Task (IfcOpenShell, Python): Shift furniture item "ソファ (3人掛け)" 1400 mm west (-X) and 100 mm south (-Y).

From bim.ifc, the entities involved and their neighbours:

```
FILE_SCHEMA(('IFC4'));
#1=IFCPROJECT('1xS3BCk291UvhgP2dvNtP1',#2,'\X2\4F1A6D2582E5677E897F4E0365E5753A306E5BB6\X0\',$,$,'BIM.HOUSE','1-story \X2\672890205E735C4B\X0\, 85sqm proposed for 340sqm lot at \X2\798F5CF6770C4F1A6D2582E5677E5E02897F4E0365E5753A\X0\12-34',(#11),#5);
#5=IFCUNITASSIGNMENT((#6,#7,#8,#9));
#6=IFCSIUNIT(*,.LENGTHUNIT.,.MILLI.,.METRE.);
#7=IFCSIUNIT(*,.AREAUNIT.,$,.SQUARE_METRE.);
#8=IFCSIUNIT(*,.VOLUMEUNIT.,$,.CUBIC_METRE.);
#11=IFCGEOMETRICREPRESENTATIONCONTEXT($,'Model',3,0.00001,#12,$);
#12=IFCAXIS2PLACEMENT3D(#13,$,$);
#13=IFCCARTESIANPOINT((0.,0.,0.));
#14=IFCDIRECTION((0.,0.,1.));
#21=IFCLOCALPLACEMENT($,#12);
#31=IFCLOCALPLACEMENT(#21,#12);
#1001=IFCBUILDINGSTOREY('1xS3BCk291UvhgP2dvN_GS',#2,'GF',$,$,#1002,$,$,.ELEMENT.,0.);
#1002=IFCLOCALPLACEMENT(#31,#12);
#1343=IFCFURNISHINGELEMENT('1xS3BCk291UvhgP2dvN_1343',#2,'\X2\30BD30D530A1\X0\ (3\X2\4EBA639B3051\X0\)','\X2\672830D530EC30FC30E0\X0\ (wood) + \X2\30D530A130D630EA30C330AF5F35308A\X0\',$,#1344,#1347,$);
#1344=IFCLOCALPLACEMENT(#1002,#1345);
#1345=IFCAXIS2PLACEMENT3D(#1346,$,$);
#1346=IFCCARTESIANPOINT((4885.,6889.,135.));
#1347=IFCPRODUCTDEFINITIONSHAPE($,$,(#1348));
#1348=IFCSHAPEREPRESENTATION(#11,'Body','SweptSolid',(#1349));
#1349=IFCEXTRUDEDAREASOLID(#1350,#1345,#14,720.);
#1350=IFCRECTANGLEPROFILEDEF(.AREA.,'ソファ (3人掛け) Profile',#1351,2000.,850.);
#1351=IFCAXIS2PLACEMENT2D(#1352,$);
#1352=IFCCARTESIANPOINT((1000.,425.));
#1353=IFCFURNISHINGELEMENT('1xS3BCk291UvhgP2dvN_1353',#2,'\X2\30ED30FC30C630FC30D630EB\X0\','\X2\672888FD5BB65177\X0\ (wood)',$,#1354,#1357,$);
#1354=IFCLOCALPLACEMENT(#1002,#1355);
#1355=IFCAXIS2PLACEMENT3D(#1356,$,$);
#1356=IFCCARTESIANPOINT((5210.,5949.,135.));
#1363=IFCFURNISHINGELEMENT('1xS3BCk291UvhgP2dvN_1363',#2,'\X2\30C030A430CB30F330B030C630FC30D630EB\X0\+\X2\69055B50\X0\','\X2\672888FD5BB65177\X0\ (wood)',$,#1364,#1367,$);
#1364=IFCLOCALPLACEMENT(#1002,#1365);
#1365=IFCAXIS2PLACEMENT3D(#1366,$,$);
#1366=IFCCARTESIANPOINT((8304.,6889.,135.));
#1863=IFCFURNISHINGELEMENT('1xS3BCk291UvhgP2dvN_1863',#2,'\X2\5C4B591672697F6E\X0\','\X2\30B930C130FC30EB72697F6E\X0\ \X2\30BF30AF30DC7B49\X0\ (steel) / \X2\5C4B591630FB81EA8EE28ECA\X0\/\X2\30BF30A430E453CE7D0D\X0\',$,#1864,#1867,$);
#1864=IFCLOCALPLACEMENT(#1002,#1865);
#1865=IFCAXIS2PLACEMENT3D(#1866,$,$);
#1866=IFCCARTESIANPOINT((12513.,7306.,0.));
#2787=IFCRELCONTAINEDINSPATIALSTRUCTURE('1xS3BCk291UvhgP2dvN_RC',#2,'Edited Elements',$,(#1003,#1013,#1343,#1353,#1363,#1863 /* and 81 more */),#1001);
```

```python
import ifcopenshell
import ifcopenshell.api.geometry
import ifcopenshell.util.placement
import ifcopenshell.util.unit

model = ifcopenshell.open("bim.ifc")
unit_scale = ifcopenshell.util.unit.calculate_unit_scale(model)

item = model.by_guid("1xS3BCk291UvhgP2dvN_1343")
matrix = ifcopenshell.util.placement.get_local_placement(item.ObjectPlacement)
matrix[0, 3] -= 1.4 / unit_scale
matrix[1, 3] -= 0.1 / unit_scale
ifcopenshell.api.geometry.edit_object_placement(model, product=item, matrix=matrix, is_si=False)

print(ifcopenshell.util.placement.get_local_placement(item.ObjectPlacement).round(3) + 0.0)

model.write("bim_v2.ifc")
```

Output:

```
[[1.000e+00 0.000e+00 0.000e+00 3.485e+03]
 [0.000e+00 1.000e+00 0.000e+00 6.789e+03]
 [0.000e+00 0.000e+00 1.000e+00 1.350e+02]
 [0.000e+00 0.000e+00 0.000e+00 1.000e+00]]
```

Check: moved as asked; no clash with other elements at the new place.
